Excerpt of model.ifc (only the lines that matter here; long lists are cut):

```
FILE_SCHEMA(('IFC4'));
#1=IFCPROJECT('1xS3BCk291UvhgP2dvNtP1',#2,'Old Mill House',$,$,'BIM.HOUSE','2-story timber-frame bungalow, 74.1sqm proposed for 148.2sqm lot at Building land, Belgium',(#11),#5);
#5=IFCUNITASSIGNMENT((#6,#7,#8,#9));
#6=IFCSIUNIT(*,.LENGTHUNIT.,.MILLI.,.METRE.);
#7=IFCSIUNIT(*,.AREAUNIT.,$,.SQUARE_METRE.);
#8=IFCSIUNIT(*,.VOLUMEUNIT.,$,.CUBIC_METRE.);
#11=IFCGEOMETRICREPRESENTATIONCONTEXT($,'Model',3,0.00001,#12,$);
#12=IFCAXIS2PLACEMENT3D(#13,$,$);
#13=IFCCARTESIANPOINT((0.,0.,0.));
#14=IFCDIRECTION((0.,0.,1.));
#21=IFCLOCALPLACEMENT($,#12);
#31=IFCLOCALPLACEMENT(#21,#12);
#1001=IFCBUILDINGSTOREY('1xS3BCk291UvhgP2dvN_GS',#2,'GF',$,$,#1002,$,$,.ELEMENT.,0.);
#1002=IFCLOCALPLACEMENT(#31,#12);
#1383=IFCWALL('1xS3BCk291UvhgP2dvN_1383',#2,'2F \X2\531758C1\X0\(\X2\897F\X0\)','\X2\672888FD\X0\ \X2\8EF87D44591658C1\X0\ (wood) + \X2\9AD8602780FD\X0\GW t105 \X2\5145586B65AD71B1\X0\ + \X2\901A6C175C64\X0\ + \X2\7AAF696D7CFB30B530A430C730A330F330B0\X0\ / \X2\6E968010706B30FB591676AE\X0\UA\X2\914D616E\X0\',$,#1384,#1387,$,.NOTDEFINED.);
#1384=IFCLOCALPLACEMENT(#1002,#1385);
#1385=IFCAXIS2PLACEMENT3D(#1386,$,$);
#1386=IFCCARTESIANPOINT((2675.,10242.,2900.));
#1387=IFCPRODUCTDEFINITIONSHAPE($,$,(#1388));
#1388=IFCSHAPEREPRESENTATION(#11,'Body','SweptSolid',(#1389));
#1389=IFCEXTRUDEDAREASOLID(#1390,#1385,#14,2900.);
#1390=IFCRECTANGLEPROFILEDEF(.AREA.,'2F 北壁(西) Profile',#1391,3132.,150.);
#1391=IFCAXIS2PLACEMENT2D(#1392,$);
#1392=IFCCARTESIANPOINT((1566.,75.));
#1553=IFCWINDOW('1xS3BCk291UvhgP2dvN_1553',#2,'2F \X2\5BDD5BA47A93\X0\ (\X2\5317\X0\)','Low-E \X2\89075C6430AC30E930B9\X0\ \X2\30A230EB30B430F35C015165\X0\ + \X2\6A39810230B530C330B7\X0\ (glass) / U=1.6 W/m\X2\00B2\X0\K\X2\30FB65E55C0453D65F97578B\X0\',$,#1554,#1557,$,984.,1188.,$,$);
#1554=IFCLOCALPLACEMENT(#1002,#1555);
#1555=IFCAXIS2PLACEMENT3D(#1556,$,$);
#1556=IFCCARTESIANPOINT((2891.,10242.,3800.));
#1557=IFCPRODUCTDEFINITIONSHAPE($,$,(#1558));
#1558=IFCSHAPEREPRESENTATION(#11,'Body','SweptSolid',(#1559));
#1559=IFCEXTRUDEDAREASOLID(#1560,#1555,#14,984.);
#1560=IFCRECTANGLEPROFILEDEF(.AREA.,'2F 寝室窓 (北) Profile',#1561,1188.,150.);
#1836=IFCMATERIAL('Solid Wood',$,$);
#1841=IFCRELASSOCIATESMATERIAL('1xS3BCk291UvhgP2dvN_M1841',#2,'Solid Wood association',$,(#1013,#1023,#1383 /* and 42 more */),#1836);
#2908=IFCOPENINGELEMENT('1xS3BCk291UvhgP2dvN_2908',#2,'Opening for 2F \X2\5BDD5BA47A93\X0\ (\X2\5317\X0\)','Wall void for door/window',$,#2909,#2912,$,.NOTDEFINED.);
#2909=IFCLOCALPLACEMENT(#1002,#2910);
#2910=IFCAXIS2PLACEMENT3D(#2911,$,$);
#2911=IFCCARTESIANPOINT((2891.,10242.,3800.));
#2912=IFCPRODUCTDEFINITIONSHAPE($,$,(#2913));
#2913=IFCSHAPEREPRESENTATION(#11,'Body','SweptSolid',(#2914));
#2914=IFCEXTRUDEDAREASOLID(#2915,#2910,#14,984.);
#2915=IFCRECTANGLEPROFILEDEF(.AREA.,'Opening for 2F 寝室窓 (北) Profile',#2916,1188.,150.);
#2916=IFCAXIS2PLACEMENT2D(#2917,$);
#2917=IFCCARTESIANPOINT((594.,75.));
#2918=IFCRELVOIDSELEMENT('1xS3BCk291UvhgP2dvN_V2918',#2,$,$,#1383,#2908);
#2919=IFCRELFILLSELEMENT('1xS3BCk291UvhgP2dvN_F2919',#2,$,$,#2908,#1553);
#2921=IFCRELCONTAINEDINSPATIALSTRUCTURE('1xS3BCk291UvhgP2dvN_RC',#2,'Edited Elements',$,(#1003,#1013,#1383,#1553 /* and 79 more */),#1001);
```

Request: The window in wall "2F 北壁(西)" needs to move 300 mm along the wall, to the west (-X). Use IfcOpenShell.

```python
import ifcopenshell
import ifcopenshell.api.geometry
import ifcopenshell.util.placement

model = ifcopenshell.open("model.ifc")

window = model.by_guid("1xS3BCk291UvhgP2dvN_1553")
opening = window.FillsVoids[0].RelatingOpeningElement
wall = opening.VoidsElements[0].RelatingBuildingElement

wall_matrix = ifcopenshell.util.placement.get_local_placement(wall.ObjectPlacement)
shift = wall_matrix[:3, 0] * -300.0
before = ifcopenshell.util.placement.get_local_placement(window.ObjectPlacement)[:3, 3].copy()

# The window is not placed relative to its opening, so move both.
for product in (opening, window):
    matrix = ifcopenshell.util.placement.get_local_placement(product.ObjectPlacement)
    matrix[:3, 3] += shift
    ifcopenshell.api.geometry.edit_object_placement(model, product=product, matrix=matrix, is_si=False)

after = ifcopenshell.util.placement.get_local_placement(window.ObjectPlacement)[:3, 3]
print("window moved by", (after - before).round(3) + 0.0)

model.write("model_edited.ifc")
```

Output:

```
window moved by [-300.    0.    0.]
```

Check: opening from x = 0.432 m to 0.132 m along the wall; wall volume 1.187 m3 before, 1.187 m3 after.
